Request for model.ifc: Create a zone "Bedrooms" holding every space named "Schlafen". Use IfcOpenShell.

First a look at what the model holds.

```python
import ifcopenshell

model = ifcopenshell.open("model.ifc")
print(model.schema)
seen = {}
for space in model.by_type("IfcSpace"):
    seen[space.LongName] = seen.get(space.LongName, 0) + 1
for name, count in sorted(seen.items(), key=str):
    print(count, "x", name)
print("zones:", [z.Name for z in model.by_type("IfcZone")][:20])
```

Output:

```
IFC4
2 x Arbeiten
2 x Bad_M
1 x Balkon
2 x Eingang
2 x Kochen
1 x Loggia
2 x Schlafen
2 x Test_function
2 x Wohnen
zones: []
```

```python
import ifcopenshell
import ifcopenshell.api.group
import ifcopenshell.api.root

model = ifcopenshell.open("model.ifc")

names = {"Schlafen"}
spaces = [s for s in model.by_type("IfcSpace") if s.LongName in names]

zone = ifcopenshell.api.root.create_entity(model, ifc_class="IfcZone", name="Bedrooms")
ifcopenshell.api.group.assign_group(model, products=spaces, group=zone)
print(len(spaces), "spaces in", zone.Name)

model.write("model_edited.ifc")
```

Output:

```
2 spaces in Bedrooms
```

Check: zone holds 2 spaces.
